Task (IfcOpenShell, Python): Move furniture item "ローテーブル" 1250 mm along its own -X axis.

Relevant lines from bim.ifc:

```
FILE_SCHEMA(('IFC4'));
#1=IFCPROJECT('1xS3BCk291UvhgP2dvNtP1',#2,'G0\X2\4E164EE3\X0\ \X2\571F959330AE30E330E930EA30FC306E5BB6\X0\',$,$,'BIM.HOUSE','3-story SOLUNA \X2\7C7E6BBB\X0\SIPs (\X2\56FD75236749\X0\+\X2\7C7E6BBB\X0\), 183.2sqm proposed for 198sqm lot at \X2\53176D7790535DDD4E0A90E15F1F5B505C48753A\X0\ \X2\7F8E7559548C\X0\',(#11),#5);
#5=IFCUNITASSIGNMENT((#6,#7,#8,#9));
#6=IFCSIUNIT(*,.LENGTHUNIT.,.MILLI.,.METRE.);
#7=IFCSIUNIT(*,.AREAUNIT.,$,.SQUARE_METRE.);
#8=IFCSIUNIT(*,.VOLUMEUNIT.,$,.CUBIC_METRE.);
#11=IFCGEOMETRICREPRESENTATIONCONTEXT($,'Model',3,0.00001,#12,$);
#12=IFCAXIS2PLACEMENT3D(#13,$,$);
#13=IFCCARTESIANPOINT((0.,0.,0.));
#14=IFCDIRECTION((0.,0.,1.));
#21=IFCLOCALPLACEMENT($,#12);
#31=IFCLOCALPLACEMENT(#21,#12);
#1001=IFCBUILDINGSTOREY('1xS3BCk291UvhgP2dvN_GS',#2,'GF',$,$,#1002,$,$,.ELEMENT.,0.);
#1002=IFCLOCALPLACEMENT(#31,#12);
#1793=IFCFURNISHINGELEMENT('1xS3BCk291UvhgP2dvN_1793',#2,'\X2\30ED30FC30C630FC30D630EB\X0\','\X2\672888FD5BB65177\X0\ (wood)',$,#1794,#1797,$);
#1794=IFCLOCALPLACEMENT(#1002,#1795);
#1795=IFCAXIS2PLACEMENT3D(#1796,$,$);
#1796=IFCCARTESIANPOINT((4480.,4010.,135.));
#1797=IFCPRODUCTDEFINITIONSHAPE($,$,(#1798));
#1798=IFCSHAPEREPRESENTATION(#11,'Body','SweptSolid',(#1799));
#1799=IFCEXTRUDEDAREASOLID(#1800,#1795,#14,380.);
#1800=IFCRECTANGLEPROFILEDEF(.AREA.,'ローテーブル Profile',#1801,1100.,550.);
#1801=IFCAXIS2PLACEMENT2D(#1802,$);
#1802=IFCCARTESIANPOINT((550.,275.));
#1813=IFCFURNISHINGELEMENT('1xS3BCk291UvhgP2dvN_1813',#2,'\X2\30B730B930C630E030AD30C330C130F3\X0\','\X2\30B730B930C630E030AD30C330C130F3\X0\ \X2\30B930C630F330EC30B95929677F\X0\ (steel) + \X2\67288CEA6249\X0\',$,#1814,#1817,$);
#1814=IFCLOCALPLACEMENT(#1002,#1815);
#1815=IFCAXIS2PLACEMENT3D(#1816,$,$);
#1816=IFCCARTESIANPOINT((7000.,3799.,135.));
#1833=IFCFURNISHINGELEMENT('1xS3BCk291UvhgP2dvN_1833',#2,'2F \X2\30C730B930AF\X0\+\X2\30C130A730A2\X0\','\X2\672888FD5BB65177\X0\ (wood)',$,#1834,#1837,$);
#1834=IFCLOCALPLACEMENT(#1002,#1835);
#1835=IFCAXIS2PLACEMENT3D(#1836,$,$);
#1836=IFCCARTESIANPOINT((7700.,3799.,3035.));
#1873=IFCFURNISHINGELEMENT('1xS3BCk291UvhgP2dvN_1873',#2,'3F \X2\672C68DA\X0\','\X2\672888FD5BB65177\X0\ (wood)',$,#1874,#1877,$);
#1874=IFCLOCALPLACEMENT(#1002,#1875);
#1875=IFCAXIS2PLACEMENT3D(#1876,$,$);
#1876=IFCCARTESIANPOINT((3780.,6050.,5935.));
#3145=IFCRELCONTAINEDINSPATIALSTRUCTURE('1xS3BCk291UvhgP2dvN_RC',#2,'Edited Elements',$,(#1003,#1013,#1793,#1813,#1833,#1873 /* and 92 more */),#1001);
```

```python
import ifcopenshell
import ifcopenshell.api.geometry
import ifcopenshell.util.placement
import ifcopenshell.util.unit

model = ifcopenshell.open("bim.ifc")
unit_scale = ifcopenshell.util.unit.calculate_unit_scale(model)

item = model.by_guid("1xS3BCk291UvhgP2dvN_1793")
matrix = ifcopenshell.util.placement.get_local_placement(item.ObjectPlacement)
matrix[:3, 3] -= matrix[:3, 0] * 1.25 / unit_scale
ifcopenshell.api.geometry.edit_object_placement(model, product=item, matrix=matrix, is_si=False)

print(ifcopenshell.util.placement.get_local_placement(item.ObjectPlacement).round(3) + 0.0)

model.write("bim_v2.ifc")
```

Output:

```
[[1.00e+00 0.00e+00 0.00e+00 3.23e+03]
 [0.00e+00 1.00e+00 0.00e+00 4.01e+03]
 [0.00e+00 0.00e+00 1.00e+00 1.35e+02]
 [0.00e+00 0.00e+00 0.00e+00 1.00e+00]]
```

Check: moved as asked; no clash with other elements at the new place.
